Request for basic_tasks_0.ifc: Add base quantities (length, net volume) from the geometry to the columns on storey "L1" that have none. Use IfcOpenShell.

First a look at what the model holds.

```python
import ifcopenshell
import ifcopenshell.util.element
import ifcopenshell.util.unit

model = ifcopenshell.open("basic_tasks_0.ifc")
print(model.schema)
for unit_type in ("LENGTHUNIT", "AREAUNIT", "VOLUMEUNIT"):
    print(unit_type, ifcopenshell.util.unit.calculate_unit_scale(model, unit_type))
storey = next(s for s in model.by_type("IfcBuildingStorey") if s.Name == "L1")
columns = [e for e in ifcopenshell.util.element.get_decomposition(storey) if e.is_a("IfcColumn")]
for e in sorted(columns, key=lambda e: e.id()):
    print(e.id(), e.is_a(), e.Name, list(ifcopenshell.util.element.get_psets(e, qtos_only=True)), sep=" | ")
```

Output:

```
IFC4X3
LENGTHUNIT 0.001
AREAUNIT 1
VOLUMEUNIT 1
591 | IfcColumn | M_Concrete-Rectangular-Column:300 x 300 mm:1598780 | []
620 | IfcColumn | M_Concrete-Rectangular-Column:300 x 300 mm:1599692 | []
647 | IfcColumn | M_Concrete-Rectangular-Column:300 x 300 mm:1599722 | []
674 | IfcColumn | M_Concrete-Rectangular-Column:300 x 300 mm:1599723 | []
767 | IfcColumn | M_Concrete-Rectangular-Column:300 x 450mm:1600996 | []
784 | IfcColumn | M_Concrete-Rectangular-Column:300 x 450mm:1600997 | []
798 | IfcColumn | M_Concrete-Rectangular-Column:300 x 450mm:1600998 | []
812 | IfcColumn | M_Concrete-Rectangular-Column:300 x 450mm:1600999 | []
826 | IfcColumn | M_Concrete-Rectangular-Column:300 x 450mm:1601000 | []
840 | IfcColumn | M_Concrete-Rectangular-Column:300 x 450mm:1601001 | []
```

```python
import ifcopenshell
import ifcopenshell.api.pset
import ifcopenshell.geom
import ifcopenshell.util.element
import ifcopenshell.util.shape
import ifcopenshell.util.unit

model = ifcopenshell.open("basic_tasks_0.ifc")
unit_scale = ifcopenshell.util.unit.calculate_unit_scale(model)
volume_scale = ifcopenshell.util.unit.calculate_unit_scale(model, "VOLUMEUNIT")
settings = ifcopenshell.geom.settings()

storey = next(s for s in model.by_type("IfcBuildingStorey") if s.Name == "L1")
columns = [e for e in ifcopenshell.util.element.get_decomposition(storey) if e.is_a("IfcColumn")]

for e in sorted(columns, key=lambda e: e.id()):
    if ifcopenshell.util.element.get_psets(e, qtos_only=True, should_inherit=False):
        continue
    # Geometry comes back in metres, in the element's own axes.
    shape = ifcopenshell.geom.create_shape(settings, e)
    values = {
        "Length": ifcopenshell.util.shape.get_z(shape.geometry) / unit_scale,
        "NetVolume": ifcopenshell.util.shape.get_volume(shape.geometry) / volume_scale,
    }
    qto = ifcopenshell.api.pset.add_qto(model, product=e, name="Qto_ColumnBaseQuantities")
    ifcopenshell.api.pset.edit_qto(model, qto=qto, properties=values)
    print(e.id(), {k: round(v, 3) for k, v in values.items()})

model.write("basic_tasks_0_updated.ifc")
```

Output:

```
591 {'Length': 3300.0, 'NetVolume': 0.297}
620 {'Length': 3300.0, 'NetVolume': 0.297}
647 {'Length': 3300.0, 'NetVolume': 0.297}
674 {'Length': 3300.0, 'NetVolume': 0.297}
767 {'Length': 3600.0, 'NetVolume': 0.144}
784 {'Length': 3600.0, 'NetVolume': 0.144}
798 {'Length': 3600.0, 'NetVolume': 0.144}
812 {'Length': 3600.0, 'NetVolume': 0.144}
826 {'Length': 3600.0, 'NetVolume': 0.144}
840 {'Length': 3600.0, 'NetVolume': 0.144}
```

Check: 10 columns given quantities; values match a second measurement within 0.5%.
